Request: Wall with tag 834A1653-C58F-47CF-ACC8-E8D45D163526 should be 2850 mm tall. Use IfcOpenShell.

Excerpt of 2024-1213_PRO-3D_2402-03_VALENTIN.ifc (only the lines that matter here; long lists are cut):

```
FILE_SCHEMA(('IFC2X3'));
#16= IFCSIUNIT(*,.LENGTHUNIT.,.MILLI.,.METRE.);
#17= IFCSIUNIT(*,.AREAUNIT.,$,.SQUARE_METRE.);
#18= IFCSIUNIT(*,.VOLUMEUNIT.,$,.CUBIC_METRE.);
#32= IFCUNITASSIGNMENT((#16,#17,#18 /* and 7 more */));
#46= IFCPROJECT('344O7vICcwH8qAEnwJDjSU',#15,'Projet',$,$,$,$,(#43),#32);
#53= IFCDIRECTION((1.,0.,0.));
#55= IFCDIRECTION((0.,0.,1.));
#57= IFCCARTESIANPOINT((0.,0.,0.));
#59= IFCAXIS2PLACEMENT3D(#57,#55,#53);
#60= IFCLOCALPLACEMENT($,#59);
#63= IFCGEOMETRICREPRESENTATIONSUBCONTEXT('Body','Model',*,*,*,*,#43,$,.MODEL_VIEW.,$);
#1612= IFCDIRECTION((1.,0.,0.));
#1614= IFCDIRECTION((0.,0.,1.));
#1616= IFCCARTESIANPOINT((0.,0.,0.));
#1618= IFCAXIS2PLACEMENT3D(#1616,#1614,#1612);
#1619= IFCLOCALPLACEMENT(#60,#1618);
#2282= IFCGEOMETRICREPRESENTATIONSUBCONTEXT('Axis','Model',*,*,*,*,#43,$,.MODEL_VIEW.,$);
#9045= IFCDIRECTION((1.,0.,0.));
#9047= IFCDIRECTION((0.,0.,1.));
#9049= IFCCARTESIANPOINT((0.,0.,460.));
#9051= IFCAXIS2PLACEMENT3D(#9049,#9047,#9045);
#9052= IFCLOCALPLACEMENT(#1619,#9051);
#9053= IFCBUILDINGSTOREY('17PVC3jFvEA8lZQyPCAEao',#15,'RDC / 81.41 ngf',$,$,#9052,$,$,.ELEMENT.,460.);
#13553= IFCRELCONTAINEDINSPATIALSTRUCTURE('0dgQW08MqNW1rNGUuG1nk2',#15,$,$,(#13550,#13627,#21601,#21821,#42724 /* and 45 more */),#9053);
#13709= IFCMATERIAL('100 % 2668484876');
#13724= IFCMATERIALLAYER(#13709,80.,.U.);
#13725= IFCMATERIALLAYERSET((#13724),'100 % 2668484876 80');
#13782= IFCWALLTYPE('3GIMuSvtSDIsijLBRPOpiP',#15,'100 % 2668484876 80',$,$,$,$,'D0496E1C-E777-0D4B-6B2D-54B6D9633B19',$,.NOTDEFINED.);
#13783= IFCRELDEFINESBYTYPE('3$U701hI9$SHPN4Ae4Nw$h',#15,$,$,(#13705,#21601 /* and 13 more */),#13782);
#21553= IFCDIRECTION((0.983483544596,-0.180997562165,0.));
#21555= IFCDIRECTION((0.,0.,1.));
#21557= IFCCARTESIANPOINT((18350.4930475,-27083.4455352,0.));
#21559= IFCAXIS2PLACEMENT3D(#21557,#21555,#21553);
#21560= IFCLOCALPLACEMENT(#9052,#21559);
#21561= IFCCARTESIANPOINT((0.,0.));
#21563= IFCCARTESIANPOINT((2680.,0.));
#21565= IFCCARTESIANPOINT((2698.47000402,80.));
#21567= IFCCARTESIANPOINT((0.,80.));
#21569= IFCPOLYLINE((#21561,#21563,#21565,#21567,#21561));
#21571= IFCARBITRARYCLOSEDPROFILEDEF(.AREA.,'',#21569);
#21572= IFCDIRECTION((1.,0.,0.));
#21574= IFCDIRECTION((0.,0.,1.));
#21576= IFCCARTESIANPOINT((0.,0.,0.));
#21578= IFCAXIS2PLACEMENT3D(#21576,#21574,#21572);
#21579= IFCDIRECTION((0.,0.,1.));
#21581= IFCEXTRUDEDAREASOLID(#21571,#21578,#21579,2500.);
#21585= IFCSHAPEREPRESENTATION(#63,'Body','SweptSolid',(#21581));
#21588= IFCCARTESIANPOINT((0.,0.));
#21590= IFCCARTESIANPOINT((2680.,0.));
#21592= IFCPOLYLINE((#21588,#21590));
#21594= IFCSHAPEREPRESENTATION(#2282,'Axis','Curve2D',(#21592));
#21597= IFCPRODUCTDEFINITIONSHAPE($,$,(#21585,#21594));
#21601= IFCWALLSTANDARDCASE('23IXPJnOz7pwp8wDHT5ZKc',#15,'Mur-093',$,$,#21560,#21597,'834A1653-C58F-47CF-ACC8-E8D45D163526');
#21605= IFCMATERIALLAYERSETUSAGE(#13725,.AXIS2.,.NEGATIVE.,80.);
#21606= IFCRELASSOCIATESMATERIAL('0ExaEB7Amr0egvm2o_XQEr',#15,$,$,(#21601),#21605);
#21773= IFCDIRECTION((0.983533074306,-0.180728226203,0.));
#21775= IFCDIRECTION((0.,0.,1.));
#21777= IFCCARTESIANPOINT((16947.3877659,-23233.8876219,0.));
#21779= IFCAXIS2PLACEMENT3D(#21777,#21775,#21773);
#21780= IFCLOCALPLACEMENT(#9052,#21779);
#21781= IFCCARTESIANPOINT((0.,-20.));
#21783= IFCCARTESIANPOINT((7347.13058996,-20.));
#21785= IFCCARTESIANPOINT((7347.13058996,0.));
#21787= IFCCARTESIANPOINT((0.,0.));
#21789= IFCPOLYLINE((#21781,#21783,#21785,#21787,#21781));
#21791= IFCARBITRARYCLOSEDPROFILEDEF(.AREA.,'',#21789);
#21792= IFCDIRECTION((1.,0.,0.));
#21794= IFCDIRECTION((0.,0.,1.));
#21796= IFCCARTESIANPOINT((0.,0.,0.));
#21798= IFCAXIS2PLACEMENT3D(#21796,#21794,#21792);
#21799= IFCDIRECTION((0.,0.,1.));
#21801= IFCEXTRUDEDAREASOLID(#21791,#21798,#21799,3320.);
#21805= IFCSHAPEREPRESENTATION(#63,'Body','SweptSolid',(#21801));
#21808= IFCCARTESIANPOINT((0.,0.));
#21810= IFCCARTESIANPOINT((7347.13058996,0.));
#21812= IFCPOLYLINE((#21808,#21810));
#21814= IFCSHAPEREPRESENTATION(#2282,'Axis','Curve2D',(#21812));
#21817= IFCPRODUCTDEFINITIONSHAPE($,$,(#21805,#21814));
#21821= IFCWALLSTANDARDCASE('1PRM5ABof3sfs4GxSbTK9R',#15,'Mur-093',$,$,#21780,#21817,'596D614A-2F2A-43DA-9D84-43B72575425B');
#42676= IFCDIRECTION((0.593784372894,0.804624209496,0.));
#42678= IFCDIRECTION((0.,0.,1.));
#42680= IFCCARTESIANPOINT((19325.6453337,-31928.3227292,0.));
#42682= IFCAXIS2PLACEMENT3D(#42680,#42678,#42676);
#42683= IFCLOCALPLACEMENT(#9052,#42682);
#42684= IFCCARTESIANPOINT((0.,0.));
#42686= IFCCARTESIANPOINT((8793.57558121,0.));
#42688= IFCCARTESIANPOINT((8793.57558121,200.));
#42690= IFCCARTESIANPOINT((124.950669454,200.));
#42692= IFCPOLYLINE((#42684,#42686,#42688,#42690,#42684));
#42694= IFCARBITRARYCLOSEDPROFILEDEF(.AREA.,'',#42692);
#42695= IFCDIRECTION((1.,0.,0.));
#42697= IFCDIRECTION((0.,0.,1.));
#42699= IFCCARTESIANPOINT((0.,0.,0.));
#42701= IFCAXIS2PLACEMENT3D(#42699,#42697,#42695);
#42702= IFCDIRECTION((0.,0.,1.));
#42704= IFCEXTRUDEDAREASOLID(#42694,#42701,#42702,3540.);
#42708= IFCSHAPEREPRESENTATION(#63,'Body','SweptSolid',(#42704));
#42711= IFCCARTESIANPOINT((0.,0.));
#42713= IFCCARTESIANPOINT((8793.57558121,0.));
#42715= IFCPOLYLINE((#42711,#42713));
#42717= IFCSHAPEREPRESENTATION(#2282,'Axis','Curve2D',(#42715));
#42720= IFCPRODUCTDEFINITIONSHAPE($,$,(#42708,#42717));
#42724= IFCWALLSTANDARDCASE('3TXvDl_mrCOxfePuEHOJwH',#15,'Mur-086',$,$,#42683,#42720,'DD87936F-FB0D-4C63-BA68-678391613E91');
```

```python
import ifcopenshell
import ifcopenshell.geom
import ifcopenshell.util.representation
import ifcopenshell.util.shape

model = ifcopenshell.open("2024-1213_PRO-3D_2402-03_VALENTIN.ifc")
settings = ifcopenshell.geom.settings()


def volume(element):
    """Net volume in cubic metres, openings subtracted."""
    shape = ifcopenshell.geom.create_shape(settings, element)
    return ifcopenshell.util.shape.get_volume(shape.geometry)


wall = model.by_id(21601)
before = volume(wall)

body = ifcopenshell.util.representation.get_representation(wall, "Model", "Body")
solid = body.Items[0]
old_height = solid.Depth
solid.Depth = 2850.0
after = volume(wall)

print(f"height {old_height:g} -> {solid.Depth:g}, volume {before:.3f} -> {after:.3f} m3")

model.write("2024-1213_PRO-3D_2402-03_VALENTIN_rev.ifc")
```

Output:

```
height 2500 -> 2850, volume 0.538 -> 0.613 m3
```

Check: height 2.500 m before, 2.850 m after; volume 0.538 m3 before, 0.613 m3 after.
